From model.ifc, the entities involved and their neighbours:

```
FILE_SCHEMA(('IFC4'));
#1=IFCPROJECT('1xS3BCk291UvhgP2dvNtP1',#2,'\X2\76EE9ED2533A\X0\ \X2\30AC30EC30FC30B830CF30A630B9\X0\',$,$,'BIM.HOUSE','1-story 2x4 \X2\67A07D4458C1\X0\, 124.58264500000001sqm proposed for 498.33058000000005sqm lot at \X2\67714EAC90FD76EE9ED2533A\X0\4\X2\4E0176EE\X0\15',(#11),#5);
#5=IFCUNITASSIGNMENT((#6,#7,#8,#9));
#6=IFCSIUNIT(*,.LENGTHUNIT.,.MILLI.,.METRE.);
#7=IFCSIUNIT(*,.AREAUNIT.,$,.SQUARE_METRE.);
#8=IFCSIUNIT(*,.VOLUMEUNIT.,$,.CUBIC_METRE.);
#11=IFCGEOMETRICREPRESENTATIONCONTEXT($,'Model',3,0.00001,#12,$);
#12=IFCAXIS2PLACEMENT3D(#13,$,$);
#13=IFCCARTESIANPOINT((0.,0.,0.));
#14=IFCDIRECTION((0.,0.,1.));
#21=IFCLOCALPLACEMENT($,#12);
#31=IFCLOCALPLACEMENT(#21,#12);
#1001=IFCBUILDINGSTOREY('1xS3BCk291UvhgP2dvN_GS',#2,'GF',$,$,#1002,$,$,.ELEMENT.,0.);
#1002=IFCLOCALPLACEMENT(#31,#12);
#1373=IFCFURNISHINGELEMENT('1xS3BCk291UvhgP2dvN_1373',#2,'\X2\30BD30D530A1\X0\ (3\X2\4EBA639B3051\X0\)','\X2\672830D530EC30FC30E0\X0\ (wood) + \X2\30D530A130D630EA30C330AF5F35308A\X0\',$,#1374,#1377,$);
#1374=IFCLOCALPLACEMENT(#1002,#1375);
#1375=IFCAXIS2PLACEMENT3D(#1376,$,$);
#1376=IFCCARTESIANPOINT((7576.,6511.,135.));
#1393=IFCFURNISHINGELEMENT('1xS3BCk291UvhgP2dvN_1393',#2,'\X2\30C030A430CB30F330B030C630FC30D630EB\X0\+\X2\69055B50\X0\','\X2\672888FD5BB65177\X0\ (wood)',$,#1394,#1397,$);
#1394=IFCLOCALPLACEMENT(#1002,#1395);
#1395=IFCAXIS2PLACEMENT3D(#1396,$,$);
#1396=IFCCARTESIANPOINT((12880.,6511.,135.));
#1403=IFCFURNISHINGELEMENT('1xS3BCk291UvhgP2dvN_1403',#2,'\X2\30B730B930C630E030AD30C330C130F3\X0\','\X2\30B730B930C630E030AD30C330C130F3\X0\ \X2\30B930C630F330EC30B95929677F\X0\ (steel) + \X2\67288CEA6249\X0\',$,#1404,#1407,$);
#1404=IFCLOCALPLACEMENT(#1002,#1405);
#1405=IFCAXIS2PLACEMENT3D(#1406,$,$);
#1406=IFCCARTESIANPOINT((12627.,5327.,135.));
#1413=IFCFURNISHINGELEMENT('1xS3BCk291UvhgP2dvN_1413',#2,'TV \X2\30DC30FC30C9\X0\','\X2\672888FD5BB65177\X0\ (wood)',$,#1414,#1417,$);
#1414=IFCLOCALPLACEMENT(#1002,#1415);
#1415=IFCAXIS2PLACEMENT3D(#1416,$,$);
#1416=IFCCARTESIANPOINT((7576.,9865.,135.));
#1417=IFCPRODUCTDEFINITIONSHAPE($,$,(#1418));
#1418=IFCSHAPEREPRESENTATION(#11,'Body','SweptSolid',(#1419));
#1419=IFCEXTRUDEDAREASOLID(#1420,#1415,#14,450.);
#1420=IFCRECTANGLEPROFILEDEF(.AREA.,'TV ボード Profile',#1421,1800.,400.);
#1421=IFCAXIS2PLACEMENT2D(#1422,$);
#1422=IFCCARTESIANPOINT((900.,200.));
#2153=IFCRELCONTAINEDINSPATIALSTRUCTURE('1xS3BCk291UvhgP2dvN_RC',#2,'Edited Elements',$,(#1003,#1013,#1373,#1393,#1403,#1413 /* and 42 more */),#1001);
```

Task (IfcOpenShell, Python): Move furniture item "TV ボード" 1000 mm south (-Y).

```python
import ifcopenshell
import ifcopenshell.api.geometry
import ifcopenshell.util.placement
import ifcopenshell.util.unit

model = ifcopenshell.open("model.ifc")
unit_scale = ifcopenshell.util.unit.calculate_unit_scale(model)

item = model.by_guid("1xS3BCk291UvhgP2dvN_1413")
matrix = ifcopenshell.util.placement.get_local_placement(item.ObjectPlacement)
matrix[1, 3] -= 1 / unit_scale
ifcopenshell.api.geometry.edit_object_placement(model, product=item, matrix=matrix, is_si=False)

print(ifcopenshell.util.placement.get_local_placement(item.ObjectPlacement).round(3) + 0.0)

model.write("model_rev.ifc")
```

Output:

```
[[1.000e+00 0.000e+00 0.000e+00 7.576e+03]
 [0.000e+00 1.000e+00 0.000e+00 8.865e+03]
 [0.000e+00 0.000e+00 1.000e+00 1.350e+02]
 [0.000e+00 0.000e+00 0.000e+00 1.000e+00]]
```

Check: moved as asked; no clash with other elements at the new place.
